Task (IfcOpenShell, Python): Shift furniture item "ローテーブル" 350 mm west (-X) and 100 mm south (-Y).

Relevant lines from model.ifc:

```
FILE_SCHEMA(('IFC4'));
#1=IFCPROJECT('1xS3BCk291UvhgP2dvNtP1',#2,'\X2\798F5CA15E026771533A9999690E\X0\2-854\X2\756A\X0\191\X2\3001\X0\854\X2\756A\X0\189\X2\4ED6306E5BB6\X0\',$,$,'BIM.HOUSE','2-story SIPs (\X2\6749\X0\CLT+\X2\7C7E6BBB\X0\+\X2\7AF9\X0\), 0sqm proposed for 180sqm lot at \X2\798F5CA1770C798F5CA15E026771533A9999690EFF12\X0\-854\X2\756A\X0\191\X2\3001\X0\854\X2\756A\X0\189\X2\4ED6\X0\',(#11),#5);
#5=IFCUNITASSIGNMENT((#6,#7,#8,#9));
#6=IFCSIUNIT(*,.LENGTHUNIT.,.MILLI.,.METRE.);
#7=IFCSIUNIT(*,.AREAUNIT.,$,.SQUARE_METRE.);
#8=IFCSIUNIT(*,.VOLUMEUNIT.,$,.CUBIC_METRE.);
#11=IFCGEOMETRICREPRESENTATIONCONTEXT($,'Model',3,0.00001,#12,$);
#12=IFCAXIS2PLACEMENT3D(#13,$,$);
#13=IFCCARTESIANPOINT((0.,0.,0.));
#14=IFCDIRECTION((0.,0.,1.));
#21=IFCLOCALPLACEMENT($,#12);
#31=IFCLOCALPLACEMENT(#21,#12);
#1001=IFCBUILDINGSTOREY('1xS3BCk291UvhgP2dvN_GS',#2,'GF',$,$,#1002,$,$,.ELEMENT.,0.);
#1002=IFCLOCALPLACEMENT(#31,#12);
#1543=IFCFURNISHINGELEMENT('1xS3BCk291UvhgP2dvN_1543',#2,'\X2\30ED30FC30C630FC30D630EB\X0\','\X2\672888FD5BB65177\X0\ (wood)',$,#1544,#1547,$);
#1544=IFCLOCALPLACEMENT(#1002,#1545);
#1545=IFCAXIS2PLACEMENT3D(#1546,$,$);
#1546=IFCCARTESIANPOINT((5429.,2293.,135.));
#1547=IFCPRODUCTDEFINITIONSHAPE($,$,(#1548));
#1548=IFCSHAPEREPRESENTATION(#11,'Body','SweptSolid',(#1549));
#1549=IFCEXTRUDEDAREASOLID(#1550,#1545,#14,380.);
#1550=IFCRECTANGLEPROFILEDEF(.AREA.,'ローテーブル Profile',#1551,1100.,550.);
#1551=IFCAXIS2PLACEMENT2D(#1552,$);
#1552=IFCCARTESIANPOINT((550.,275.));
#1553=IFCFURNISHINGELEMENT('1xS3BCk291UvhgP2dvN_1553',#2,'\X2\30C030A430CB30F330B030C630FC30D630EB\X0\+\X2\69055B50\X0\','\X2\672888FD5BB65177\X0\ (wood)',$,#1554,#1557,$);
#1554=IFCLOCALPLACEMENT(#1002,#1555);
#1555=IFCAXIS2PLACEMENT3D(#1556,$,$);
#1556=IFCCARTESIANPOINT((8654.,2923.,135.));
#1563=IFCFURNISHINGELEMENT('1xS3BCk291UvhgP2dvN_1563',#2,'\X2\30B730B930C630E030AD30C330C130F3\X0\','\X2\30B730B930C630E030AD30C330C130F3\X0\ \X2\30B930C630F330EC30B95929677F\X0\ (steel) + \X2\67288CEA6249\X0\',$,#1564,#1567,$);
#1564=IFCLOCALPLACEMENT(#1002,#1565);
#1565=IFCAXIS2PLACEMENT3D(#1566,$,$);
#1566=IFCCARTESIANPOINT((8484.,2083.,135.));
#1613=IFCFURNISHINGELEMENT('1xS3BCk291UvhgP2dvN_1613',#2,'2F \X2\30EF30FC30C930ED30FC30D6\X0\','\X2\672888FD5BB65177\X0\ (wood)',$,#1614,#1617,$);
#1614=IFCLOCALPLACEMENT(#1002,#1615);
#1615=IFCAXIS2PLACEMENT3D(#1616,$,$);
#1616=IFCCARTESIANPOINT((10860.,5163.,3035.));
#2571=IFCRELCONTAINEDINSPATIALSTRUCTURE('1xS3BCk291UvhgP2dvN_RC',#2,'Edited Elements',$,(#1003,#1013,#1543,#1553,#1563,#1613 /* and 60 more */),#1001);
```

```python
import ifcopenshell
import ifcopenshell.api.geometry
import ifcopenshell.util.placement

model = ifcopenshell.open("model.ifc")

item = model.by_guid("1xS3BCk291UvhgP2dvN_1543")
matrix = ifcopenshell.util.placement.get_local_placement(item.ObjectPlacement)
matrix[0, 3] -= 350.0
matrix[1, 3] -= 100.0
ifcopenshell.api.geometry.edit_object_placement(model, product=item, matrix=matrix, is_si=False)

print(ifcopenshell.util.placement.get_local_placement(item.ObjectPlacement).round(3) + 0.0)

model.write("model_updated.ifc")
```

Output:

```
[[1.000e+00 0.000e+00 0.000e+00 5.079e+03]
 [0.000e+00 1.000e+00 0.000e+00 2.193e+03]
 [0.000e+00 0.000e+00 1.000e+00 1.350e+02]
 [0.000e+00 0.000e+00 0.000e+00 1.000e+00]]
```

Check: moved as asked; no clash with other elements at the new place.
